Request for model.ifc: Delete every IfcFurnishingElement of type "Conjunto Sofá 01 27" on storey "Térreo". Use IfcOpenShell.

First a look at what the model holds.

```python
import ifcopenshell
import ifcopenshell.util.element

model = ifcopenshell.open("model.ifc")
print(model.schema)
storey = next(s for s in model.by_type("IfcBuildingStorey") if s.Name == "Térreo")
furniture = [e for e in ifcopenshell.util.element.get_decomposition(storey) if e.is_a("IfcFurnishingElement")]
seen = {}
for e in furniture:
    element_type = ifcopenshell.util.element.get_type(e)
    name = element_type.Name if element_type not in (None, e) else None
    seen[name] = seen.get(name, 0) + 1
for name, count in sorted(seen.items(), key=str):
    print(count, "x", name)
```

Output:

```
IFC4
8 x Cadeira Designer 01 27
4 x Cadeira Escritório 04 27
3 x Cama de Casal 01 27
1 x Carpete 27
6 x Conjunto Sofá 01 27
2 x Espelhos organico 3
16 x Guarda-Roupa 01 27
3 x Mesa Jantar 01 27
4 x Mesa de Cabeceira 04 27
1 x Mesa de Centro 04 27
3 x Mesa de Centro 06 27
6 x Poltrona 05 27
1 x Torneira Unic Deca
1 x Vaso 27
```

```python
import ifcopenshell
import ifcopenshell.api.root
import ifcopenshell.util.element

model = ifcopenshell.open("model.ifc")

storey = next(s for s in model.by_type("IfcBuildingStorey") if s.Name == "Térreo")
furniture = [e for e in ifcopenshell.util.element.get_decomposition(storey) if e.is_a("IfcFurnishingElement")]
targets = [e for e in furniture if (t := ifcopenshell.util.element.get_type(e)) not in (None, e) and t.Name == "Conjunto Sofá 01 27"]

for e in targets:
    ifcopenshell.api.root.remove_product(model, product=e)
print(len(targets), "removed")

model.write("model_v2.ifc")
```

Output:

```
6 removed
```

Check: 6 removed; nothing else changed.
